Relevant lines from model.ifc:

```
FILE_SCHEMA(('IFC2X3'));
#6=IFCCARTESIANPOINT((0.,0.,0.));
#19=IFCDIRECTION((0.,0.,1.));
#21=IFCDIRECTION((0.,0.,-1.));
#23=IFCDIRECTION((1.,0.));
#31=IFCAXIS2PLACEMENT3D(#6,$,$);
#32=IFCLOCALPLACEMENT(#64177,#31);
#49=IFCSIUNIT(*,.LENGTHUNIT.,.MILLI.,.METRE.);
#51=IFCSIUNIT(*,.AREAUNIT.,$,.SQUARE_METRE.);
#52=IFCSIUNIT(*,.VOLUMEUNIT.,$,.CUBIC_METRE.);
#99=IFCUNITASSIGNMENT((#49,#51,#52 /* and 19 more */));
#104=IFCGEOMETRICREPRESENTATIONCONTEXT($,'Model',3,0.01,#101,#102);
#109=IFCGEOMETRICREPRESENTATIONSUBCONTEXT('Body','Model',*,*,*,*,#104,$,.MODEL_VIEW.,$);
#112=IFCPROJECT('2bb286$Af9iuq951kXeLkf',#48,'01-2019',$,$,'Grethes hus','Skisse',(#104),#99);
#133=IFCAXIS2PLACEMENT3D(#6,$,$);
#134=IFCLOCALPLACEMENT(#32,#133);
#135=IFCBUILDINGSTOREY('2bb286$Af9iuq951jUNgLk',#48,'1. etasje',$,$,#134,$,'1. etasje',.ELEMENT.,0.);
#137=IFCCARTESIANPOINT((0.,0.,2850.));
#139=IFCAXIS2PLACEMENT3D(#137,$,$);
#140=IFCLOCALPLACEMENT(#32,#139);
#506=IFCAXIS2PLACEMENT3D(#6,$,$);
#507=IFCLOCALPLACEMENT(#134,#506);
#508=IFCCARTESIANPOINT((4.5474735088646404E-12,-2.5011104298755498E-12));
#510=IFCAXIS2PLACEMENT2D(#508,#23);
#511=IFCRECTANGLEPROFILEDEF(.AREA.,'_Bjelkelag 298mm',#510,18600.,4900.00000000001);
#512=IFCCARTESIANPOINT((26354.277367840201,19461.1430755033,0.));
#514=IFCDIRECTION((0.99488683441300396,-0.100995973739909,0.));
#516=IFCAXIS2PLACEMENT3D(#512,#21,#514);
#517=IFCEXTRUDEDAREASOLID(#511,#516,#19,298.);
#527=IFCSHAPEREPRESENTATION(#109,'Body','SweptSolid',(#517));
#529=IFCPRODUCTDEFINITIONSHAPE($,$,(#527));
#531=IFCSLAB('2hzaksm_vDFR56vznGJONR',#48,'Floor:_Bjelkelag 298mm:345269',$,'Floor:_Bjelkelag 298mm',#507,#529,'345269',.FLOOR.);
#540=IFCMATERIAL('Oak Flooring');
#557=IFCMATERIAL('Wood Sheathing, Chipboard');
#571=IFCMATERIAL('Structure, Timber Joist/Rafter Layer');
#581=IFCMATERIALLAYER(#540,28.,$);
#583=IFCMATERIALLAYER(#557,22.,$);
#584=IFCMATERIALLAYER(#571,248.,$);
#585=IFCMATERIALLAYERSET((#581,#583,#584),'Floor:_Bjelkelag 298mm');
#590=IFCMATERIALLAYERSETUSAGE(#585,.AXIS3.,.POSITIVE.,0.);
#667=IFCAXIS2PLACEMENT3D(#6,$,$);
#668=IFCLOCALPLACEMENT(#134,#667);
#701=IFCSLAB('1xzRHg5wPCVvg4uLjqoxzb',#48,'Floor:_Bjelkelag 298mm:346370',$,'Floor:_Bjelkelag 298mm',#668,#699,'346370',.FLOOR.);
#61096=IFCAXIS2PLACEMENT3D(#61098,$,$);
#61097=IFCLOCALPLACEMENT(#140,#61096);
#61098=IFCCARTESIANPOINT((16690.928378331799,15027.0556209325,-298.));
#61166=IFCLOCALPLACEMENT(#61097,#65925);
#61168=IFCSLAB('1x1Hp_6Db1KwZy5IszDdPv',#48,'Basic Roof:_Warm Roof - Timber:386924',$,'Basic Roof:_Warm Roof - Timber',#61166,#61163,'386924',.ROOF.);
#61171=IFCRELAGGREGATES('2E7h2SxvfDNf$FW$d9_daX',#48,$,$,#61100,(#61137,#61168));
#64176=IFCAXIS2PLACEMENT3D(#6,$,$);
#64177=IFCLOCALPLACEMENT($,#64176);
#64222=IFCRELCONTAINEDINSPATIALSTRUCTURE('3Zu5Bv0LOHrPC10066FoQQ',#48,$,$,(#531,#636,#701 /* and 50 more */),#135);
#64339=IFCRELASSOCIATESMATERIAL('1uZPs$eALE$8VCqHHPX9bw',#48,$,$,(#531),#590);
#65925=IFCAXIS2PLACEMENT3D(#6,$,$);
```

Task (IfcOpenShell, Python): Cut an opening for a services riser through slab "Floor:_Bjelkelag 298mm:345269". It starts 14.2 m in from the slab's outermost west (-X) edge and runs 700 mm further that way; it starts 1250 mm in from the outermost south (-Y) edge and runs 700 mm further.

```python
import numpy as np
import ifcopenshell
import ifcopenshell.api.feature
import ifcopenshell.api.geometry
import ifcopenshell.api.root
import ifcopenshell.geom
import ifcopenshell.util.placement
import ifcopenshell.util.representation
import ifcopenshell.util.shape
import ifcopenshell.util.unit

model = ifcopenshell.open("model.ifc")
unit_scale = ifcopenshell.util.unit.calculate_unit_scale(model)
settings = ifcopenshell.geom.settings()


def volume(element):
    """Net volume in cubic metres, openings subtracted."""
    shape = ifcopenshell.geom.create_shape(settings, element)
    return ifcopenshell.util.shape.get_volume(shape.geometry)


slab = model.by_id(531)
before = volume(slab)

# Extent in the slab's own axes, in metres. The edges named are its -X and -Y sides.
slab_shape = ifcopenshell.geom.create_shape(settings, slab)
vertices = ifcopenshell.util.shape.get_vertices(slab_shape.geometry)
x_min, y_min, bottom = vertices.min(axis=0)
top = vertices[:, 2].max()

opening = ifcopenshell.api.root.create_entity(model, ifc_class="IfcOpeningElement", name="Services riser opening")
context = ifcopenshell.util.representation.get_context(model, "Model", "Body", "MODEL_VIEW")
width, depth = 0.7, 0.7
outline = [(0.0, 0.0), (width, 0.0), (width, depth), (0.0, depth), (0.0, 0.0)]
# Overshoot both faces by 50 mm so the cut is clean.
shape = ifcopenshell.api.geometry.add_slab_representation(
    model, context=context, depth=top - bottom + 0.1, polyline=outline
)
ifcopenshell.api.geometry.assign_representation(model, product=opening, representation=shape)

matrix = ifcopenshell.util.placement.get_local_placement(slab.ObjectPlacement)
matrix[:, 3] = matrix @ np.append(np.array([x_min + 14.2, y_min + 1.25, bottom - 0.05]) / unit_scale, 1.0)
ifcopenshell.api.geometry.edit_object_placement(model, product=opening, matrix=matrix, is_si=False)
ifcopenshell.api.feature.add_feature(model, feature=opening, element=slab)

after = volume(slab)

print(f"slab volume {before:.3f} -> {after:.3f} m3")

model.write("model_v2.ifc")
```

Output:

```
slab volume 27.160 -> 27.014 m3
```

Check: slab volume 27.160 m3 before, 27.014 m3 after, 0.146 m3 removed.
